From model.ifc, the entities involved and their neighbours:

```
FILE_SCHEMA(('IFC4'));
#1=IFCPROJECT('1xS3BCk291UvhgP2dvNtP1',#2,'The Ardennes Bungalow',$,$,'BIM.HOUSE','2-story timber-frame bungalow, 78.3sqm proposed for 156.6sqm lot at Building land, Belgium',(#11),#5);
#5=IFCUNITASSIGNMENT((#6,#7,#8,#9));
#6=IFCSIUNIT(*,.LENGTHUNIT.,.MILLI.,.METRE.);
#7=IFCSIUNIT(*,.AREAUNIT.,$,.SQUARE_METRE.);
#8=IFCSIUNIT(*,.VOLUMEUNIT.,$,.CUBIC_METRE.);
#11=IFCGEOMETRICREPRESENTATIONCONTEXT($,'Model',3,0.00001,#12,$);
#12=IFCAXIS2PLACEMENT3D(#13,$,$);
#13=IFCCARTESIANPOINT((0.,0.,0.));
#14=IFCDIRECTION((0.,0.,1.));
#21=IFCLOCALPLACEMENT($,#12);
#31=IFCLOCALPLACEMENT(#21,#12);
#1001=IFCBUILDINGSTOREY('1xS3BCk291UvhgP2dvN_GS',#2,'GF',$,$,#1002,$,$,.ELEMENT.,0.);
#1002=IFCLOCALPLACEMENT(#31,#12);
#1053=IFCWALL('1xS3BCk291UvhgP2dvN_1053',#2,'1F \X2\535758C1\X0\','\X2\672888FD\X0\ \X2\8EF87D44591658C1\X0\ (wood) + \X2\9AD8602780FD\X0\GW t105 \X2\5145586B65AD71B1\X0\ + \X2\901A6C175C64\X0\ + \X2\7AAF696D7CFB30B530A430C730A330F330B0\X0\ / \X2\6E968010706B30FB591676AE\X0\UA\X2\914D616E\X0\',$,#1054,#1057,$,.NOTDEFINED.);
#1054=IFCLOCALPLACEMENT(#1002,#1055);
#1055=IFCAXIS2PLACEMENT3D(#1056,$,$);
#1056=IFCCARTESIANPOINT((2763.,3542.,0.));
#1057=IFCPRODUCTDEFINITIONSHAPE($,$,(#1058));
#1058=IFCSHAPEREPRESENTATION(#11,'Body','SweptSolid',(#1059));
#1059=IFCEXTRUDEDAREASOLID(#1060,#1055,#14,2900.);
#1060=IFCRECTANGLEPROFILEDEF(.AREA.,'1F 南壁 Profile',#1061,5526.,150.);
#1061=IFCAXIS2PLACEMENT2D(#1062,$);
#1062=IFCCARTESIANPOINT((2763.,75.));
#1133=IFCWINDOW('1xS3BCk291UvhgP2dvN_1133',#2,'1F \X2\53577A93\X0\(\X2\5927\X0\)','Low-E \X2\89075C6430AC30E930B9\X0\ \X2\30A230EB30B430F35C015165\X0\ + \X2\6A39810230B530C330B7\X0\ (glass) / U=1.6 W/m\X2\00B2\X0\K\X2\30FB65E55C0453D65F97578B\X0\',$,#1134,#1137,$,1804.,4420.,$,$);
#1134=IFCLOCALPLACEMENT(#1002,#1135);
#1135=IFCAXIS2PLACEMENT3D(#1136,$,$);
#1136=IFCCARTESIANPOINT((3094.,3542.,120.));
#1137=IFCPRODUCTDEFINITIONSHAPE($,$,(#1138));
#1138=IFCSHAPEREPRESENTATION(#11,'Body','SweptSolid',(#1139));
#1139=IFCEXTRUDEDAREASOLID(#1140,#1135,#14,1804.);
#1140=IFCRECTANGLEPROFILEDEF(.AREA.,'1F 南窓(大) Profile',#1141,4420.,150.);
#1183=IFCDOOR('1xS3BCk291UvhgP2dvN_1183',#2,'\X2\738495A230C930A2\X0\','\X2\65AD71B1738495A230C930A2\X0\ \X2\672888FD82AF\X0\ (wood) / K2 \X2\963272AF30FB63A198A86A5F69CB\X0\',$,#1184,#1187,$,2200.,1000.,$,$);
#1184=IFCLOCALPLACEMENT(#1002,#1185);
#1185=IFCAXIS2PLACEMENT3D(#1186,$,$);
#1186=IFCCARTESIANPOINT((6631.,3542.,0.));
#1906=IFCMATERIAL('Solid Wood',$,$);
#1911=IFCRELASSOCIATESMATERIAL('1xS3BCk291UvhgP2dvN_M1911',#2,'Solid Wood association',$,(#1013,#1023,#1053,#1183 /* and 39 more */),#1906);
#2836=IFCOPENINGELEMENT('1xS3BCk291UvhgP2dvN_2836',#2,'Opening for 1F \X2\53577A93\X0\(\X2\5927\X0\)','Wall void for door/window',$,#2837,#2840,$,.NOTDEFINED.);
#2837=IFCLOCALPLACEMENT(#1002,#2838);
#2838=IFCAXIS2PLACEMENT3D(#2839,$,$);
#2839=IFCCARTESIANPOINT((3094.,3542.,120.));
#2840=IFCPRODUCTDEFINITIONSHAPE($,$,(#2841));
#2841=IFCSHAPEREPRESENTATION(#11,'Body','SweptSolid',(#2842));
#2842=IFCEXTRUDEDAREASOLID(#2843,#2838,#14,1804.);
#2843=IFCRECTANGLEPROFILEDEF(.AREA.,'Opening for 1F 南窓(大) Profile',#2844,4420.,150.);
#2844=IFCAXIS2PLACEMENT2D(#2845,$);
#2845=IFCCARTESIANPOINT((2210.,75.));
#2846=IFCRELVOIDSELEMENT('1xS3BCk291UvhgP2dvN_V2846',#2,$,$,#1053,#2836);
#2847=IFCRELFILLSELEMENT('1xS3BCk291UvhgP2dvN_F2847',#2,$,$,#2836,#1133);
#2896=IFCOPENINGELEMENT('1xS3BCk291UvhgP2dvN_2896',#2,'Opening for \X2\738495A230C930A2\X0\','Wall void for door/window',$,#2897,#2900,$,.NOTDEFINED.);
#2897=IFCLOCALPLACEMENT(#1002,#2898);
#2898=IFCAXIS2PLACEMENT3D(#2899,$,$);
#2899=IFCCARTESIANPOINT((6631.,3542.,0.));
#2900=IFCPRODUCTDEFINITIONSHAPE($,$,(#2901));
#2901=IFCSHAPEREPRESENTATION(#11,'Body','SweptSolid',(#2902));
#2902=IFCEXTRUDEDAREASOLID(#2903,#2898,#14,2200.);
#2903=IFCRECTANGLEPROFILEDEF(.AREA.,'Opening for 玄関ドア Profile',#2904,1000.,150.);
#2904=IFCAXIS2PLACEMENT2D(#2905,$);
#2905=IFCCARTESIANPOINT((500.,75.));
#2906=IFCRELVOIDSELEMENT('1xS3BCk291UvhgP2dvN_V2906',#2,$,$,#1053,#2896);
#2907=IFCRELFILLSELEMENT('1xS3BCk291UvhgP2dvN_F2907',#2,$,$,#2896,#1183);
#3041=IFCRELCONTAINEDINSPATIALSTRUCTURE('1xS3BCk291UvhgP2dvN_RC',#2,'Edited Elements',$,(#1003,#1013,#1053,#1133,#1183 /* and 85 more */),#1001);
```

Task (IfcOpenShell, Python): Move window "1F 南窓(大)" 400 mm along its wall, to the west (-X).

```python
import ifcopenshell
import ifcopenshell.api.geometry
import ifcopenshell.util.placement

model = ifcopenshell.open("model.ifc")

window = model.by_guid("1xS3BCk291UvhgP2dvN_1133")
opening = window.FillsVoids[0].RelatingOpeningElement
wall = opening.VoidsElements[0].RelatingBuildingElement

wall_matrix = ifcopenshell.util.placement.get_local_placement(wall.ObjectPlacement)
shift = wall_matrix[:3, 0] * -400.0
before = ifcopenshell.util.placement.get_local_placement(window.ObjectPlacement)[:3, 3].copy()

# The window is not placed relative to its opening, so move both.
for product in (opening, window):
    matrix = ifcopenshell.util.placement.get_local_placement(product.ObjectPlacement)
    matrix[:3, 3] += shift
    ifcopenshell.api.geometry.edit_object_placement(model, product=product, matrix=matrix, is_si=False)

after = ifcopenshell.util.placement.get_local_placement(window.ObjectPlacement)[:3, 3]
print("window moved by", (after - before).round(3) + 0.0)

model.write("model_edited.ifc")
```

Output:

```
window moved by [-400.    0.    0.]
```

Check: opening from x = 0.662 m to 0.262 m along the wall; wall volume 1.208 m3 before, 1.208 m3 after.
